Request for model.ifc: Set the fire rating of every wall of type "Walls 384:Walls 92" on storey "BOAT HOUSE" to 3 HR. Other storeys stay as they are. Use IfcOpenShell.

First a look at what the model holds.

```python
import ifcopenshell
import ifcopenshell.util.element

model = ifcopenshell.open("model.ifc")
print(model.schema)
storey = next(s for s in model.by_type("IfcBuildingStorey") if s.Name == "BOAT HOUSE")
walls = [e for e in ifcopenshell.util.element.get_decomposition(storey) if e.is_a("IfcWall")]
seen = {}
for e in walls:
    element_type = ifcopenshell.util.element.get_type(e)
    key = (element_type.Name if element_type != e and element_type else None, ifcopenshell.util.element.get_pset(e, "Pset_WallCommon", "FireRating"))
    seen[key] = seen.get(key, 0) + 1
for (name, value), count in sorted(seen.items(), key=str):
    print(count, "x", name, "|", value)
```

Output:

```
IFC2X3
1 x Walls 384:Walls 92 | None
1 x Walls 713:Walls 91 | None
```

```python
import ifcopenshell
import ifcopenshell.api.pset
import ifcopenshell.util.element

model = ifcopenshell.open("model.ifc")

storey = next(s for s in model.by_type("IfcBuildingStorey") if s.Name == "BOAT HOUSE")
walls = [e for e in ifcopenshell.util.element.get_decomposition(storey) if e.is_a("IfcWall")]

count = 0
for e in walls:
    element_type = ifcopenshell.util.element.get_type(e)
    if element_type in (None, e) or element_type.Name != "Walls 384:Walls 92":
        continue
    # add_pset returns the element's existing set when there is one.
    pset = ifcopenshell.api.pset.add_pset(model, product=e, name="Pset_WallCommon")
    ifcopenshell.api.pset.edit_pset(model, pset=pset, properties={"FireRating": "3 HR"})
    count += 1

print(count, "walls updated")

model.write("model-out.ifc")
```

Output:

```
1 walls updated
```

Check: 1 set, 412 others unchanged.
